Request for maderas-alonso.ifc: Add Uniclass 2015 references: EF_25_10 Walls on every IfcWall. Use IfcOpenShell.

First a look at what the model holds.

```python
import ifcopenshell

model = ifcopenshell.open("maderas-alonso.ifc")
print(model.schema)
print("classifications:", [c.Name for c in model.by_type("IfcClassification")])
for ifc_class in ("IfcDoor", "IfcRoof", "IfcStair", "IfcWall", "IfcWindow"):
    print(ifc_class, len(model.by_type(ifc_class)))
```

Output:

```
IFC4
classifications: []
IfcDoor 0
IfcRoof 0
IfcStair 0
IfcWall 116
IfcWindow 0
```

```python
import ifcopenshell
import ifcopenshell.api.classification

model = ifcopenshell.open("maderas-alonso.ifc")

system = ifcopenshell.api.classification.add_classification(model, classification="Uniclass 2015")

codes = {
    "IfcWall": ("EF_25_10", "Walls"),
}
for ifc_class, (code, name) in codes.items():
    products = model.by_type(ifc_class)
    ifcopenshell.api.classification.add_reference(
        model, products=products, classification=system, identification=code, name=name
    )
    print(code, len(products))

model.write("maderas-alonso_v2.ifc")
```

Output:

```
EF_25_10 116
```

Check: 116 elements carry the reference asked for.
